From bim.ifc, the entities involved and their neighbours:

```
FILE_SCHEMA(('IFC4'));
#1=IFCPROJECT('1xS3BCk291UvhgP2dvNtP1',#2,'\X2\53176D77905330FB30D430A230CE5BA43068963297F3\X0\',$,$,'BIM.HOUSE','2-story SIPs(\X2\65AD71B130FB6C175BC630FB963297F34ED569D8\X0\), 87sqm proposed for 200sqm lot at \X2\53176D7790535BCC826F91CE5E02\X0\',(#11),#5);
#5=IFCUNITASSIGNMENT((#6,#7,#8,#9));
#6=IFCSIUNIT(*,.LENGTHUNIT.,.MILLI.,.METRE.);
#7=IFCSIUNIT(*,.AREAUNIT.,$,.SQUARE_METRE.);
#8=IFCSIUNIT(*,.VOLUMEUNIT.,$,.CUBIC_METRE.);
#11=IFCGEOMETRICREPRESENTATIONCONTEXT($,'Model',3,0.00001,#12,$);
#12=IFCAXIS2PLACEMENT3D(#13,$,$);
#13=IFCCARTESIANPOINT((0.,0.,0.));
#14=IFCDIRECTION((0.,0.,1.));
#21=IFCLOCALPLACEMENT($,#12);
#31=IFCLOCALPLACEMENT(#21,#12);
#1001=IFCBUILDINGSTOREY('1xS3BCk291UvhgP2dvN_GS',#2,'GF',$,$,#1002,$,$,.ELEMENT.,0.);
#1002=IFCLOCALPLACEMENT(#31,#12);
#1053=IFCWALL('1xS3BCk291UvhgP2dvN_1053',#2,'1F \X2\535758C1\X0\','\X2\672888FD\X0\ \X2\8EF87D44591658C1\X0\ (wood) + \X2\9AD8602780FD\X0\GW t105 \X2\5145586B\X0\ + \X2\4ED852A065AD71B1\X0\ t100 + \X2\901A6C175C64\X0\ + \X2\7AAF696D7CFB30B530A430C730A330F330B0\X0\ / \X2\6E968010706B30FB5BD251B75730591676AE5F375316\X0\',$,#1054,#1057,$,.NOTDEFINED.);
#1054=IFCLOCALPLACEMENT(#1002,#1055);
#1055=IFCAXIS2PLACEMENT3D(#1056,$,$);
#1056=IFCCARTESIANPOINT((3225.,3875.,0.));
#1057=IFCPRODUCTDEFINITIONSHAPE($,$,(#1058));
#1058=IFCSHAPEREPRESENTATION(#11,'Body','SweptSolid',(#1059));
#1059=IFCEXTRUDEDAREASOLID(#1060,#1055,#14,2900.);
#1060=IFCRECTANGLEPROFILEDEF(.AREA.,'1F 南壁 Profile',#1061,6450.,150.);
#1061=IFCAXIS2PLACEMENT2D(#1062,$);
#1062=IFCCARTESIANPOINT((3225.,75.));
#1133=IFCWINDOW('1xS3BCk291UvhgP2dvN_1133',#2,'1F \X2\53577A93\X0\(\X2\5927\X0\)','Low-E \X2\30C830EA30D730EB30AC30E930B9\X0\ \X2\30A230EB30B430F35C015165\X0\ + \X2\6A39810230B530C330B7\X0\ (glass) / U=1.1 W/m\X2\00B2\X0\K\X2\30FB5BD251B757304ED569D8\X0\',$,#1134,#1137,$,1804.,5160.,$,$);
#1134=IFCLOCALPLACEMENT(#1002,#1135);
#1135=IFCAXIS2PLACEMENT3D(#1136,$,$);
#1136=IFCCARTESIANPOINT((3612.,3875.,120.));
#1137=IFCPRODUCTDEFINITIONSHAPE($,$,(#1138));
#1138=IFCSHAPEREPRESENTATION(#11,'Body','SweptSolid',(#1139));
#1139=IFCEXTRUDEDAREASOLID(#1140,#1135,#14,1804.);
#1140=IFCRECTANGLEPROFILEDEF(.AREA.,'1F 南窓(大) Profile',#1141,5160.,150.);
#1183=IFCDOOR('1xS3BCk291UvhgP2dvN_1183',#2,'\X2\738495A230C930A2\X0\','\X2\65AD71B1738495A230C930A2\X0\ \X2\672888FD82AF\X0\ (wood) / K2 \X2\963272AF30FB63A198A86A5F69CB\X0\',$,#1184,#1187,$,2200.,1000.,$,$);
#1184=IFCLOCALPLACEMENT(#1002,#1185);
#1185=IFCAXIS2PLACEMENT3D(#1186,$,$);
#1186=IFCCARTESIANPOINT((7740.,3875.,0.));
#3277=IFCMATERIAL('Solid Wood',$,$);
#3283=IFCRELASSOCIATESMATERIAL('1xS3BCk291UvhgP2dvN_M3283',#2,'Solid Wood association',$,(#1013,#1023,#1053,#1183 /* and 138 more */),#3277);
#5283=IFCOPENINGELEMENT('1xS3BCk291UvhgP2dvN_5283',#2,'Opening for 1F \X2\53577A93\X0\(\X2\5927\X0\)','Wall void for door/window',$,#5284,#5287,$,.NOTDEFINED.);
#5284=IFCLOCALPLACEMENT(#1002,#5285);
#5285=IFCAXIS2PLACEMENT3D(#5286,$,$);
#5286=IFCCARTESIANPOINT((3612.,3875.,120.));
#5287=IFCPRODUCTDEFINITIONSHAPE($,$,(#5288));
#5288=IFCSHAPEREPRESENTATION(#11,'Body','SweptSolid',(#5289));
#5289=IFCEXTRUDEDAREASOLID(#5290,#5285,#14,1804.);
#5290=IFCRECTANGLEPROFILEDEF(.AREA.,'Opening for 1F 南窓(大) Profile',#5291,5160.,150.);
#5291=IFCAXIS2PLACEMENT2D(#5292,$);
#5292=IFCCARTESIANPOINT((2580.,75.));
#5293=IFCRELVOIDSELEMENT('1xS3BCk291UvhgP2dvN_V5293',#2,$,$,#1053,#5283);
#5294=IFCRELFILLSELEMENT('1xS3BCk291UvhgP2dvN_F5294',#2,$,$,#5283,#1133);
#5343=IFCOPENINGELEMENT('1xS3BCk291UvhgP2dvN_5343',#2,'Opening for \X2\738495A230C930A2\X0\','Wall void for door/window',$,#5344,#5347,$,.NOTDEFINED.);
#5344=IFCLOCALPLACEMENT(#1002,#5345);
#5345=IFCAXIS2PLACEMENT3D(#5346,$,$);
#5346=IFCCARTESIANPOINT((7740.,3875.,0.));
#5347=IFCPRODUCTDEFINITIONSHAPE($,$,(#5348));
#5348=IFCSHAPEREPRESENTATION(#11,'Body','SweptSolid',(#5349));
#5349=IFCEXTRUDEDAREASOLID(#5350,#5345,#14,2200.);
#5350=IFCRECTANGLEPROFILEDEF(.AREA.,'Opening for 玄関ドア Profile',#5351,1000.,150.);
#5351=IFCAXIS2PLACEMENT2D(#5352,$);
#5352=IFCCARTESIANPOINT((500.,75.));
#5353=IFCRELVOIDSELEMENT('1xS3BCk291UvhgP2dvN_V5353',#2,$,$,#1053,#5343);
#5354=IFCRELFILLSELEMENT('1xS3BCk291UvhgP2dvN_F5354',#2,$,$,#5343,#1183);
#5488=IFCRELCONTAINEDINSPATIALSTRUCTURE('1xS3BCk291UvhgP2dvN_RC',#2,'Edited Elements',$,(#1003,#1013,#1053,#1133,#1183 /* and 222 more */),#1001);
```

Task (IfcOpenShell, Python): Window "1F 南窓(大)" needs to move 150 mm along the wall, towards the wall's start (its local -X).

```python
import ifcopenshell
import ifcopenshell.api.geometry
import ifcopenshell.util.placement
import ifcopenshell.util.unit

model = ifcopenshell.open("bim.ifc")
unit_scale = ifcopenshell.util.unit.calculate_unit_scale(model)

window = model.by_guid("1xS3BCk291UvhgP2dvN_1133")
opening = window.FillsVoids[0].RelatingOpeningElement
wall = opening.VoidsElements[0].RelatingBuildingElement

wall_matrix = ifcopenshell.util.placement.get_local_placement(wall.ObjectPlacement)
shift = wall_matrix[:3, 0] * -0.15 / unit_scale
before = ifcopenshell.util.placement.get_local_placement(window.ObjectPlacement)[:3, 3].copy()

# The window is not placed relative to its opening, so move both.
for product in (opening, window):
    matrix = ifcopenshell.util.placement.get_local_placement(product.ObjectPlacement)
    matrix[:3, 3] += shift
    ifcopenshell.api.geometry.edit_object_placement(model, product=product, matrix=matrix, is_si=False)

after = ifcopenshell.util.placement.get_local_placement(window.ObjectPlacement)[:3, 3]
print("window moved by", (after - before).round(3) + 0.0)

model.write("bim_rev.ifc")
```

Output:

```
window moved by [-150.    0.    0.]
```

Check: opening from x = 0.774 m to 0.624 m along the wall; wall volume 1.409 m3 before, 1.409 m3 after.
